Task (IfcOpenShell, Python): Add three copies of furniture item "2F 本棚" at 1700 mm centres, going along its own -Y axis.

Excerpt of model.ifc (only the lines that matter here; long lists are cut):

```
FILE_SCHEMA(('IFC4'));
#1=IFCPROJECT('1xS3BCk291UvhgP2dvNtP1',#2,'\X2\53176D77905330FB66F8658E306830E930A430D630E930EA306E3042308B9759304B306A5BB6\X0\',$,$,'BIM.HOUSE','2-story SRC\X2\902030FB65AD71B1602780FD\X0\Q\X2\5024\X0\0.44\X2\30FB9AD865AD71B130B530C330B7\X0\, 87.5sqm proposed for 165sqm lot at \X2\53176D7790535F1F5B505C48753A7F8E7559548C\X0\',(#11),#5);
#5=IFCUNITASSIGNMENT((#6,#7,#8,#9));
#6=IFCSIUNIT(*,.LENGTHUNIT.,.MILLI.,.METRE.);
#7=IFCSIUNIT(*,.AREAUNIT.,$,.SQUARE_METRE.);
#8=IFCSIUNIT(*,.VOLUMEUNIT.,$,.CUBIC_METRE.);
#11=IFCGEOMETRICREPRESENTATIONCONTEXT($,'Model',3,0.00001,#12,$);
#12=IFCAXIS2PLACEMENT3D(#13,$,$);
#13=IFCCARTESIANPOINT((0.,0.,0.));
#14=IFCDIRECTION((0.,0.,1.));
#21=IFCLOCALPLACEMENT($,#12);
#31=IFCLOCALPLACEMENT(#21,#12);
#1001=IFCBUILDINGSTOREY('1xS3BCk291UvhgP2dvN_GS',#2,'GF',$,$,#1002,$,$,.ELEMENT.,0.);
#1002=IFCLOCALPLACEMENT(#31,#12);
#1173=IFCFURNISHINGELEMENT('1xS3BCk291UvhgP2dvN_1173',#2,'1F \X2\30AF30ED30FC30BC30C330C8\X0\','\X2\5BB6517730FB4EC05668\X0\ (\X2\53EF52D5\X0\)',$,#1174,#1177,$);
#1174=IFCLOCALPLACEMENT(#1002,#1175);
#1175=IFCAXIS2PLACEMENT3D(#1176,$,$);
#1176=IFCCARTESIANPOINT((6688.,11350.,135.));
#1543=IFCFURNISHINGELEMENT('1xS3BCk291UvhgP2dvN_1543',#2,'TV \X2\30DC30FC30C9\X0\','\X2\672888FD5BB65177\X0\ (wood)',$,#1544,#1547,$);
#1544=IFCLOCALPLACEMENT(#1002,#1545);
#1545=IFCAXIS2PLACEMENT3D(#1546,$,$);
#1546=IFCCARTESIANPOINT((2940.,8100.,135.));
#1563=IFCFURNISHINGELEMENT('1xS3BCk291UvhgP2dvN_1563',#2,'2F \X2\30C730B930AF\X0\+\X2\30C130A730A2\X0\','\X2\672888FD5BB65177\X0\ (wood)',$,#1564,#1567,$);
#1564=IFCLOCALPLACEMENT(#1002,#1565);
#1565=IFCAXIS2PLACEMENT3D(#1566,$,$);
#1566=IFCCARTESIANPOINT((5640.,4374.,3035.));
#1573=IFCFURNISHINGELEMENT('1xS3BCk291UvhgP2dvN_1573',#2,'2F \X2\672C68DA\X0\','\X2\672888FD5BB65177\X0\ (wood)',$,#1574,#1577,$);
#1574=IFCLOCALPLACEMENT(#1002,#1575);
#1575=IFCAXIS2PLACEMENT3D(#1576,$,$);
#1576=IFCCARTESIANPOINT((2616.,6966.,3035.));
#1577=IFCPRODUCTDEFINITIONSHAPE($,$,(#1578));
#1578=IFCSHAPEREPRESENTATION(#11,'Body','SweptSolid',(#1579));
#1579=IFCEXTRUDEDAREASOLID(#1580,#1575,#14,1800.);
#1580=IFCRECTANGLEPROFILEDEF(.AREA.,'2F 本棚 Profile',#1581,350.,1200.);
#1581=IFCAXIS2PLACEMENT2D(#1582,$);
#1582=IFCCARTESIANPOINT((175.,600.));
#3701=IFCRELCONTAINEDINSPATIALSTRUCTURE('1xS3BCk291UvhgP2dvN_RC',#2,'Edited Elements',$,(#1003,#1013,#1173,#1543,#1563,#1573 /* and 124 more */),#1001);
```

```python
import ifcopenshell
import ifcopenshell.api.geometry
import ifcopenshell.api.root
import ifcopenshell.util.element
import ifcopenshell.util.placement

model = ifcopenshell.open("model.ifc")


def reuse_history(source, copy):
    """copy_class also copies each property set's owner history, people and application; keep the originals."""
    for rel in copy.IsDefinedBy:
        if rel.is_a("IfcRelDefinesByProperties") and (history := rel.RelatingPropertyDefinition.OwnerHistory):
            rel.RelatingPropertyDefinition.OwnerHistory = source.OwnerHistory
            ifcopenshell.util.element.remove_deep2(model, history)


source = model.by_id(1573)
base = ifcopenshell.util.placement.get_local_placement(source.ObjectPlacement)
step = -base[:3, 1] * 1700.0

for i in range(1, 4):
    copy = ifcopenshell.api.root.copy_class(model, product=source)
    copy.Representation = ifcopenshell.util.element.copy_deep(
        model, source.Representation, exclude=["IfcGeometricRepresentationContext", "IfcRepresentationMap"]
    )
    reuse_history(source, copy)
    matrix = base.copy()
    matrix[:3, 3] += i * step
    print("added at", matrix[:3, 3].round(3) + 0.0)
    ifcopenshell.api.geometry.edit_object_placement(model, product=copy, matrix=matrix, is_si=False)

model.write("model_edited.ifc")
```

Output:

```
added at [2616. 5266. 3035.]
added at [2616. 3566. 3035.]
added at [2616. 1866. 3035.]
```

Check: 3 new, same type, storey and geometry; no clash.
